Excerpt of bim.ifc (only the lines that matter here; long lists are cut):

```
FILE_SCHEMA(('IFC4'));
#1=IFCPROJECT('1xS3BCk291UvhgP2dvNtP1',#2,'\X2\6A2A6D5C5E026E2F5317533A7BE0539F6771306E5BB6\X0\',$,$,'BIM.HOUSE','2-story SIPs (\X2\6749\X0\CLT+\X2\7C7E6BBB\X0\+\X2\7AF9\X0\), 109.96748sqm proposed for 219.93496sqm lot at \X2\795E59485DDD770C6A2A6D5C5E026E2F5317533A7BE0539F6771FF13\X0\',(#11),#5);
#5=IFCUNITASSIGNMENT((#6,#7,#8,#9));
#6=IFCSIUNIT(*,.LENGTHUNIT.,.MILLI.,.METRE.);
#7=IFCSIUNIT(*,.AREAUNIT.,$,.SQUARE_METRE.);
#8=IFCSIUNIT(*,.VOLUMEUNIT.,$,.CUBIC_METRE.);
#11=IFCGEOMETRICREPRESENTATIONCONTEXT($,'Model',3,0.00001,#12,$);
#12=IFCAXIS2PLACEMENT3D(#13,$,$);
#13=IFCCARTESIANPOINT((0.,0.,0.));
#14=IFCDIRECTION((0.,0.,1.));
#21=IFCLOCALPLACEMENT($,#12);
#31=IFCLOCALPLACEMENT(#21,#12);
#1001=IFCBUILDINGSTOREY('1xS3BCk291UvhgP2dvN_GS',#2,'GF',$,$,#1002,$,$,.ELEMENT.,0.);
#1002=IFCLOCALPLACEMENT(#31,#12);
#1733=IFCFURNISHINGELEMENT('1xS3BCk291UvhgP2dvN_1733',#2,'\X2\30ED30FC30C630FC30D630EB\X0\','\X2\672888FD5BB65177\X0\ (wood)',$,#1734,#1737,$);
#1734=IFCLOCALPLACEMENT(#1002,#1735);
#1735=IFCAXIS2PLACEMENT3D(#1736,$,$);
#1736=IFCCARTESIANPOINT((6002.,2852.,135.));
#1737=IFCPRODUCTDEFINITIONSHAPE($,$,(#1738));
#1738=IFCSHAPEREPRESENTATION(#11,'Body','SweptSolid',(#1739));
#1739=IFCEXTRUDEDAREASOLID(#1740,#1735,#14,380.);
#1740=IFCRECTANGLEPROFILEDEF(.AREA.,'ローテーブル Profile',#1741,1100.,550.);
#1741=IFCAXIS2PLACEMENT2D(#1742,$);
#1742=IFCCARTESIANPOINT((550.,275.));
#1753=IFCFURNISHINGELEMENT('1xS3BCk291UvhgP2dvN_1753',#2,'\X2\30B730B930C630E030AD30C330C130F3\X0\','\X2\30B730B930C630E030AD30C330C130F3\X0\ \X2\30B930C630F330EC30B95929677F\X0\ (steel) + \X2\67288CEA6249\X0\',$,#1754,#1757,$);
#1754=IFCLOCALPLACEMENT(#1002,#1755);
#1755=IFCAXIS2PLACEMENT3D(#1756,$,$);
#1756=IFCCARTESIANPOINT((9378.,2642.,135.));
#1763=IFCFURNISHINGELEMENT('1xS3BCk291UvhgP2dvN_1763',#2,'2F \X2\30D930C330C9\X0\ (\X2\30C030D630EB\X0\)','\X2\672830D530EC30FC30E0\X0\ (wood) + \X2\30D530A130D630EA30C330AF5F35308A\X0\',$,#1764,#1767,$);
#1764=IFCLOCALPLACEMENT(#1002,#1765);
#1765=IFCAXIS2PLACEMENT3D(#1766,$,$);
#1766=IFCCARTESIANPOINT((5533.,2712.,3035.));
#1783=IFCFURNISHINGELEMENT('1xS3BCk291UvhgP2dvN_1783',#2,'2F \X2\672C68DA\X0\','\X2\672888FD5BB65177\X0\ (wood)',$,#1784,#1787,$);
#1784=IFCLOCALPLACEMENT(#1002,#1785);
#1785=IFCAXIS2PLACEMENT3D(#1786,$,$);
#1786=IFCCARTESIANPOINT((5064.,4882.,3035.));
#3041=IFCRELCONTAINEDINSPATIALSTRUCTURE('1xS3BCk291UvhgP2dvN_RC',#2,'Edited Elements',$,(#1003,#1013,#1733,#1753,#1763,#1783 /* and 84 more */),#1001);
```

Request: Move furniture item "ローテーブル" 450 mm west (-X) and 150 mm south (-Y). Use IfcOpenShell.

```python
import ifcopenshell
import ifcopenshell.api.geometry
import ifcopenshell.util.placement
import ifcopenshell.util.unit

model = ifcopenshell.open("bim.ifc")
unit_scale = ifcopenshell.util.unit.calculate_unit_scale(model)

item = model.by_id(1733)
matrix = ifcopenshell.util.placement.get_local_placement(item.ObjectPlacement)
matrix[0, 3] -= 0.45 / unit_scale
matrix[1, 3] -= 0.15 / unit_scale
ifcopenshell.api.geometry.edit_object_placement(model, product=item, matrix=matrix, is_si=False)

print(ifcopenshell.util.placement.get_local_placement(item.ObjectPlacement).round(3) + 0.0)

model.write("bim_v2.ifc")
```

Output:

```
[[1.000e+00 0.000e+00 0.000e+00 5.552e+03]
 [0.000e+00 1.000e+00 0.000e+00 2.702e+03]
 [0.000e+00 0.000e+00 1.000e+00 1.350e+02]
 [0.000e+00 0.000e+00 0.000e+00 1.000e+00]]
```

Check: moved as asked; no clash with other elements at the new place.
